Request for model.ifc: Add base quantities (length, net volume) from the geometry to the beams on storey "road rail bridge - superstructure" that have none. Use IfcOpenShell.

First a look at what the model holds.

```python
import ifcopenshell
import ifcopenshell.util.element
import ifcopenshell.util.unit

model = ifcopenshell.open("model.ifc")
print(model.schema)
for unit_type in ("LENGTHUNIT", "AREAUNIT", "VOLUMEUNIT"):
    print(unit_type, ifcopenshell.util.unit.calculate_unit_scale(model, unit_type))
storey = next(s for s in model.by_type("IfcBuildingStorey") if s.Name == "road rail bridge - superstructure")
beams = [e for e in ifcopenshell.util.element.get_decomposition(storey) if e.is_a("IfcBeam")]
for e in sorted(beams, key=lambda e: e.id()):
    print(e.id(), e.is_a(), e.Name, list(ifcopenshell.util.element.get_psets(e, qtos_only=True)), sep=" | ")
```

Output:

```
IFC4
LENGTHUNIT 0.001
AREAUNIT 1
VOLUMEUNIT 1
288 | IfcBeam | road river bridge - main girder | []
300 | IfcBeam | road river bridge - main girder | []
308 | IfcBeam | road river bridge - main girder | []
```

```python
import ifcopenshell
import ifcopenshell.api.pset
import ifcopenshell.geom
import ifcopenshell.util.element
import ifcopenshell.util.shape
import ifcopenshell.util.unit

model = ifcopenshell.open("model.ifc")
unit_scale = ifcopenshell.util.unit.calculate_unit_scale(model)
volume_scale = ifcopenshell.util.unit.calculate_unit_scale(model, "VOLUMEUNIT")
settings = ifcopenshell.geom.settings()

storey = next(s for s in model.by_type("IfcBuildingStorey") if s.Name == "road rail bridge - superstructure")
beams = [e for e in ifcopenshell.util.element.get_decomposition(storey) if e.is_a("IfcBeam")]

for e in sorted(beams, key=lambda e: e.id()):
    if ifcopenshell.util.element.get_psets(e, qtos_only=True, should_inherit=False):
        continue
    # Geometry comes back in metres, in the element's own axes.
    shape = ifcopenshell.geom.create_shape(settings, e)
    values = {
        "Length": ifcopenshell.util.shape.get_max_xyz(shape.geometry) / unit_scale,
        "NetVolume": ifcopenshell.util.shape.get_volume(shape.geometry) / volume_scale,
    }
    qto = ifcopenshell.api.pset.add_qto(model, product=e, name="Qto_BeamBaseQuantities")
    ifcopenshell.api.pset.edit_qto(model, qto=qto, properties=values)
    print(e.id(), {k: round(v, 3) for k, v in values.items()})

model.write("model-out.ifc")
```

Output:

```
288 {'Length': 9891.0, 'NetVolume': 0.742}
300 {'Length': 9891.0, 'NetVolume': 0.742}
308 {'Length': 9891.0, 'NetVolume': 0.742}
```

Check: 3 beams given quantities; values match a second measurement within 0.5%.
